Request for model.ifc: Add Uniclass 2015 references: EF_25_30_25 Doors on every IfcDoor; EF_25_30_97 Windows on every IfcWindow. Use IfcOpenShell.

First a look at what the model holds.

```python
import ifcopenshell

model = ifcopenshell.open("model.ifc")
print(model.schema)
print("classifications:", [c.Name for c in model.by_type("IfcClassification")])
for ifc_class in ("IfcDoor", "IfcRoof", "IfcStair", "IfcWall", "IfcWindow"):
    print(ifc_class, len(model.by_type(ifc_class)))
```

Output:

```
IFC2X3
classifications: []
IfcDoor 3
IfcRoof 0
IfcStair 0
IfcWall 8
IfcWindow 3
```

```python
import ifcopenshell
import ifcopenshell.api.classification

model = ifcopenshell.open("model.ifc")

# IFC2X3 requires Source and Edition and has no link from the project to the system.
system = model.create_entity("IfcClassification", Source="NBS", Edition="2015", Name="Uniclass 2015")

codes = {
    "IfcDoor": ("EF_25_30_25", "Doors"),
    "IfcWindow": ("EF_25_30_97", "Windows"),
}
for ifc_class, (code, name) in codes.items():
    products = model.by_type(ifc_class)
    ifcopenshell.api.classification.add_reference(
        model, products=products, classification=system, identification=code, name=name
    )
    print(code, len(products))

model.write("model-out.ifc")
```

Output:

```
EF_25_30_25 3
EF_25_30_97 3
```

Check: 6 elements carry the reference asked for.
